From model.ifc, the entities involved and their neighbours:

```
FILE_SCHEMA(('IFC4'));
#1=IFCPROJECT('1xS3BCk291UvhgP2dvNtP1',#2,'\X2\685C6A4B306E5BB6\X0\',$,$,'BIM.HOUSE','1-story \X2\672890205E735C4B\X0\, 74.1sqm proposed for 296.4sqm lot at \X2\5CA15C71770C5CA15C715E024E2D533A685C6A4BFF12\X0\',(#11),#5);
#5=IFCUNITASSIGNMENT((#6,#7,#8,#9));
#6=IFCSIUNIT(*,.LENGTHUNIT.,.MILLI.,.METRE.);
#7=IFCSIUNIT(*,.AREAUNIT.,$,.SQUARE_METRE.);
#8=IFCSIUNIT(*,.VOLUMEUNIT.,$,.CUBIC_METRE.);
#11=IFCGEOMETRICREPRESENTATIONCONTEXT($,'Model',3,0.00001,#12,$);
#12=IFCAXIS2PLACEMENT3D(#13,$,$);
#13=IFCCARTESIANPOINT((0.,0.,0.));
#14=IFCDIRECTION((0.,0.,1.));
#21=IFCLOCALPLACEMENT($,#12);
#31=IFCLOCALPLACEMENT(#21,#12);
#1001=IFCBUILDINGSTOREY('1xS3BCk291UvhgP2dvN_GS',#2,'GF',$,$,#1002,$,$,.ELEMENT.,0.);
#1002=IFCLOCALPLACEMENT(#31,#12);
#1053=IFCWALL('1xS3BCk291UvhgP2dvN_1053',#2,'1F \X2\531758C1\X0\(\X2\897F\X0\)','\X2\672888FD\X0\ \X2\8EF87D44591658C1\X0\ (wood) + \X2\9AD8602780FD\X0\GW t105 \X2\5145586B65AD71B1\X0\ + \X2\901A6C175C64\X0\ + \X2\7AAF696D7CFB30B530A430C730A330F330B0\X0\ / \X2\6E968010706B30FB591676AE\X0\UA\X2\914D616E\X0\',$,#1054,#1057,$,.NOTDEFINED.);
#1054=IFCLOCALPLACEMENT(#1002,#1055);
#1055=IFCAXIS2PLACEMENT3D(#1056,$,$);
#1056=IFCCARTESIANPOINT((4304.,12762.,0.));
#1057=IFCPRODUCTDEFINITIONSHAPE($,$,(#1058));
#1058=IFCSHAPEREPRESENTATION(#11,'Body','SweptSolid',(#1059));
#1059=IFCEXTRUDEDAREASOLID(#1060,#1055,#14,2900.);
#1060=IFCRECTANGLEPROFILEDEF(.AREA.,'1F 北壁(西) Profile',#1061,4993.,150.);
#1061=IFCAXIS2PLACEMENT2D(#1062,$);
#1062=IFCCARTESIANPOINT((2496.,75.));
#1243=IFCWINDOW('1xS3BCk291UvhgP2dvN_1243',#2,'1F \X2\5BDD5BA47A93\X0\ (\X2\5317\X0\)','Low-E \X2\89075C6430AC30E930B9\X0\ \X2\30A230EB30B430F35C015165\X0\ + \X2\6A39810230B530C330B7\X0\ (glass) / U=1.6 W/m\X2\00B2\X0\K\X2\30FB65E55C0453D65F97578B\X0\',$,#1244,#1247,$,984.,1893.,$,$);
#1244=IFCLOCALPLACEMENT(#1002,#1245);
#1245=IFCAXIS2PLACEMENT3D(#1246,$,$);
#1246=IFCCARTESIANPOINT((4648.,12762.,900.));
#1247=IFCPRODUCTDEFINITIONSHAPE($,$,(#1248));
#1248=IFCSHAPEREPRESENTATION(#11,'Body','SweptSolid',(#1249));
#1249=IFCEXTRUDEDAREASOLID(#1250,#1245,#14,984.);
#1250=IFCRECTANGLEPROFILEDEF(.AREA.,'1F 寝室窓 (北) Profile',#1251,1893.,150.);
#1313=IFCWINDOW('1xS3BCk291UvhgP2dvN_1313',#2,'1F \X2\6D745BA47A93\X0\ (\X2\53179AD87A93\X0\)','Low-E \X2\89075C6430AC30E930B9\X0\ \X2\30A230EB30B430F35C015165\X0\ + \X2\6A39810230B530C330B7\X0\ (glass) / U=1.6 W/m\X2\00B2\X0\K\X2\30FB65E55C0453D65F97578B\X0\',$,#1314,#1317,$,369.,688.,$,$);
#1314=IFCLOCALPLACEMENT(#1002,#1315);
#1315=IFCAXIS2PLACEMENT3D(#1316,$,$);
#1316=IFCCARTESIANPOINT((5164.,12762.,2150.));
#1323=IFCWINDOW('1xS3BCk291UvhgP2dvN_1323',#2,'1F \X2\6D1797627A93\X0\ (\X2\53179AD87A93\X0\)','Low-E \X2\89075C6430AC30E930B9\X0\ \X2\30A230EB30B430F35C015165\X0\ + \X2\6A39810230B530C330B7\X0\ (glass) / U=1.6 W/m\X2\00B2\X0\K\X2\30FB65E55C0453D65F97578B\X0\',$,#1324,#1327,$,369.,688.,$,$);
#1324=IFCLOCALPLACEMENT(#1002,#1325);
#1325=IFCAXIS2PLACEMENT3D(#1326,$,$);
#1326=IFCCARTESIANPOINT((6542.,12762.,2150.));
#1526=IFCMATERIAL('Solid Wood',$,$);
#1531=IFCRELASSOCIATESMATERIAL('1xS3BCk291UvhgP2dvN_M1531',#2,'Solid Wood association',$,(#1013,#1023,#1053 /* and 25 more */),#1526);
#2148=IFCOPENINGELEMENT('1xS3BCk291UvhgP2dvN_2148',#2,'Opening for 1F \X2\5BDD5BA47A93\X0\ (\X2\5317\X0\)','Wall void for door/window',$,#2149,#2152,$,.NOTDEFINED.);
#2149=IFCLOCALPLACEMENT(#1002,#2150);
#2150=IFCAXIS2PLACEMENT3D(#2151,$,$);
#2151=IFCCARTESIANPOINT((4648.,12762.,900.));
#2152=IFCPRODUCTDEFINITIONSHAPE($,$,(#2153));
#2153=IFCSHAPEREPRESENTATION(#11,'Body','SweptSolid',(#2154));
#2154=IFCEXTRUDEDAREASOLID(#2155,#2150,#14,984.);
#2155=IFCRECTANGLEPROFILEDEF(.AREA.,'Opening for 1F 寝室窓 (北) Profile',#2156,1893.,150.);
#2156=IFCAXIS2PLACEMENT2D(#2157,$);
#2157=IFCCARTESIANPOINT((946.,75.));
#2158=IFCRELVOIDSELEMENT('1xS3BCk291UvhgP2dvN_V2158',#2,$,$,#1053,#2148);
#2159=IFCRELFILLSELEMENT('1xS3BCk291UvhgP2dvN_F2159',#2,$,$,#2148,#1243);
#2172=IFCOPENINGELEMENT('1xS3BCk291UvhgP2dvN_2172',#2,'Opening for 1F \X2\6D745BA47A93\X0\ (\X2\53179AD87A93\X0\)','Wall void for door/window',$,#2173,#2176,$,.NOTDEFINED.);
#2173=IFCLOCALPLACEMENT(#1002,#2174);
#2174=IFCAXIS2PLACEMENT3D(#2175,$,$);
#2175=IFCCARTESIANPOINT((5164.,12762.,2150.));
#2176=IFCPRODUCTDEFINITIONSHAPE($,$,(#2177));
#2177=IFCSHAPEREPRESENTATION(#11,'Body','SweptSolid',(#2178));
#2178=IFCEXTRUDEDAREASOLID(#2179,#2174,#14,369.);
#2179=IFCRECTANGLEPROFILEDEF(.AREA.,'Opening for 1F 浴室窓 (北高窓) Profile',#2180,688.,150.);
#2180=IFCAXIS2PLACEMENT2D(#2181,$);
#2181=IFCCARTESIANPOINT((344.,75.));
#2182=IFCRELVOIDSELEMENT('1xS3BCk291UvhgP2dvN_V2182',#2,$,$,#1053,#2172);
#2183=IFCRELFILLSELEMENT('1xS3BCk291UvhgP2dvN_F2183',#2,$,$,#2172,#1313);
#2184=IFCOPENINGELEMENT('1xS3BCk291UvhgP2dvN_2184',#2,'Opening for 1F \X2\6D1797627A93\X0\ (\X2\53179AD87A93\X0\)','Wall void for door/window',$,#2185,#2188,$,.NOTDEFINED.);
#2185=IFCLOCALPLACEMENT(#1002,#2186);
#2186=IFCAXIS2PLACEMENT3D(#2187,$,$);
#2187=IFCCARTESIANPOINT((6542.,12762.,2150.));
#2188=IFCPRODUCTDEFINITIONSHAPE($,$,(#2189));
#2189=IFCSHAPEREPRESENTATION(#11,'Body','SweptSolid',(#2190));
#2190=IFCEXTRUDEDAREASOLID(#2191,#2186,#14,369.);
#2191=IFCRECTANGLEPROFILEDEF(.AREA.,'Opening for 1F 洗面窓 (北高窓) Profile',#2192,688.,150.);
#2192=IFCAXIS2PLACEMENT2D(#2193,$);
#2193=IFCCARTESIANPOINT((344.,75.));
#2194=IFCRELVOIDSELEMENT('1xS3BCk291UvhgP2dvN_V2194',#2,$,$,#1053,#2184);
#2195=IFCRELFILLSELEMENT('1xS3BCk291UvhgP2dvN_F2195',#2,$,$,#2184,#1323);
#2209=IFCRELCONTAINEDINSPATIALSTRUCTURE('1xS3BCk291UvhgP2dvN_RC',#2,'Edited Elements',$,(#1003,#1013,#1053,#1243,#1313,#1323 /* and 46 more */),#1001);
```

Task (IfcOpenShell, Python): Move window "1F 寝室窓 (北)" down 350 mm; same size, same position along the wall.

```python
import numpy as np
import ifcopenshell
import ifcopenshell.api.geometry
import ifcopenshell.util.placement
import ifcopenshell.util.unit

model = ifcopenshell.open("model.ifc")
unit_scale = ifcopenshell.util.unit.calculate_unit_scale(model)

window = model.by_guid("1xS3BCk291UvhgP2dvN_1243")
opening = window.FillsVoids[0].RelatingOpeningElement
dz = -350.0

shift = np.array([0.0, 0.0, dz])
# The window is not placed relative to its opening, so move both.
for product in (opening, window):
    matrix = ifcopenshell.util.placement.get_local_placement(product.ObjectPlacement)
    matrix[:3, 3] += shift
    ifcopenshell.api.geometry.edit_object_placement(model, product=product, matrix=matrix, is_si=False)

print(f"moved by {dz * unit_scale:+.3f} m")

model.write("model-out.ifc")
```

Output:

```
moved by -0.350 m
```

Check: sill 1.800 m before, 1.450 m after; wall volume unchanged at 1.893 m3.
